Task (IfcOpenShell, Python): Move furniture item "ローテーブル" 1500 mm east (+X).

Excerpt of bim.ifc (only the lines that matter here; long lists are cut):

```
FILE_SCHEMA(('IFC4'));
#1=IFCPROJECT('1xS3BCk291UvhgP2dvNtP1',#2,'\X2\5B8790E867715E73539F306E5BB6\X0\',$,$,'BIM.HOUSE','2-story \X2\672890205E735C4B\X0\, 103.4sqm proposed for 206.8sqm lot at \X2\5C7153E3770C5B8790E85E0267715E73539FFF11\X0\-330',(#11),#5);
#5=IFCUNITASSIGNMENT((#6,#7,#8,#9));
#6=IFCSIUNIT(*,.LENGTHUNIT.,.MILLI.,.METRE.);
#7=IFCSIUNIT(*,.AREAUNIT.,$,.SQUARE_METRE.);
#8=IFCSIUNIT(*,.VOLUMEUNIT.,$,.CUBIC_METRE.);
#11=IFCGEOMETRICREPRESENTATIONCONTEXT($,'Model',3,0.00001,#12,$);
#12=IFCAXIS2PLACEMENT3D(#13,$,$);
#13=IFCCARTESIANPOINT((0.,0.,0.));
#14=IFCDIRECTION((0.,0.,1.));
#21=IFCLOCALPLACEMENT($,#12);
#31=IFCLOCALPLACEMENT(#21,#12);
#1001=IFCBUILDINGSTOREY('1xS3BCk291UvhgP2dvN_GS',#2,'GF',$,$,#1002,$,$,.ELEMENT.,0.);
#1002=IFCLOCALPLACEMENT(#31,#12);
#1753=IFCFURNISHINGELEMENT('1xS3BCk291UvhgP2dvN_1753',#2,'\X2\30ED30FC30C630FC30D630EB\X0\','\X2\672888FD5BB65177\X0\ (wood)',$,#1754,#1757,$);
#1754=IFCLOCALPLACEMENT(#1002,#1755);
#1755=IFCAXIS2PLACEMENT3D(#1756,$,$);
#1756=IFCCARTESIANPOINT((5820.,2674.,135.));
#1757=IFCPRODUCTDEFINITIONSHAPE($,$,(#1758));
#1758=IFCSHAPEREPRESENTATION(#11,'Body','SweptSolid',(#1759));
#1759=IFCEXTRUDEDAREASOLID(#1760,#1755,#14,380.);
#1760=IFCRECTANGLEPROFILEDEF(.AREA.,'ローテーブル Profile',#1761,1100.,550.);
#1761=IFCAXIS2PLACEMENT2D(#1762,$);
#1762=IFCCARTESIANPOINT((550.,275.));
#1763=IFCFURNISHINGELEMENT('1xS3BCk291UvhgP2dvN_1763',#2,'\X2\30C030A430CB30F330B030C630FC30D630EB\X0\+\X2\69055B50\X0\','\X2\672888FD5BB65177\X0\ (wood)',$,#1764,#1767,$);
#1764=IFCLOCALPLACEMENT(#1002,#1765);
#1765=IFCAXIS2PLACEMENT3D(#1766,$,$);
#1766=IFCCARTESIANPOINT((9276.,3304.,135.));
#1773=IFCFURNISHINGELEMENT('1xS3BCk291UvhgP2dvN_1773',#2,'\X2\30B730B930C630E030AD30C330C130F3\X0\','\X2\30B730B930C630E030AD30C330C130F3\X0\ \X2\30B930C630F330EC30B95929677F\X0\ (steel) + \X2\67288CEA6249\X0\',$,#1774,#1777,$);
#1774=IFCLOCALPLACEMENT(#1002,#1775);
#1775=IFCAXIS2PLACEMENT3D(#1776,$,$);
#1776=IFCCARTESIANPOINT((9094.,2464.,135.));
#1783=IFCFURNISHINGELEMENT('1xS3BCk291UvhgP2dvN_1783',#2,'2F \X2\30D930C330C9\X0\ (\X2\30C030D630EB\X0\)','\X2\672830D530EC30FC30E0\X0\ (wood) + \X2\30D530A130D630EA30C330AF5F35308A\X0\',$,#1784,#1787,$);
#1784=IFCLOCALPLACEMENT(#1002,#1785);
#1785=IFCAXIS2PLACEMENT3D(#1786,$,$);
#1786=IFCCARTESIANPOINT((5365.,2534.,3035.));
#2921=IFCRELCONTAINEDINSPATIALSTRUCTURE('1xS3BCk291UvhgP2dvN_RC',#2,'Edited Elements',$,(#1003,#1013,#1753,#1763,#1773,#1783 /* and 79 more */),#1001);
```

```python
import ifcopenshell
import ifcopenshell.api.geometry
import ifcopenshell.util.placement

model = ifcopenshell.open("bim.ifc")

item = model.by_guid("1xS3BCk291UvhgP2dvN_1753")
matrix = ifcopenshell.util.placement.get_local_placement(item.ObjectPlacement)
matrix[0, 3] += 1500.0
ifcopenshell.api.geometry.edit_object_placement(model, product=item, matrix=matrix, is_si=False)

print(ifcopenshell.util.placement.get_local_placement(item.ObjectPlacement).round(3) + 0.0)

model.write("bim_v2.ifc")
```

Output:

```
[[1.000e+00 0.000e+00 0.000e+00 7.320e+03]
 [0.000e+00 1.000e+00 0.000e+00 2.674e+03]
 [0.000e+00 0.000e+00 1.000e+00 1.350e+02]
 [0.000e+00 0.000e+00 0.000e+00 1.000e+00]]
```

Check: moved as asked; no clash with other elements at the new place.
